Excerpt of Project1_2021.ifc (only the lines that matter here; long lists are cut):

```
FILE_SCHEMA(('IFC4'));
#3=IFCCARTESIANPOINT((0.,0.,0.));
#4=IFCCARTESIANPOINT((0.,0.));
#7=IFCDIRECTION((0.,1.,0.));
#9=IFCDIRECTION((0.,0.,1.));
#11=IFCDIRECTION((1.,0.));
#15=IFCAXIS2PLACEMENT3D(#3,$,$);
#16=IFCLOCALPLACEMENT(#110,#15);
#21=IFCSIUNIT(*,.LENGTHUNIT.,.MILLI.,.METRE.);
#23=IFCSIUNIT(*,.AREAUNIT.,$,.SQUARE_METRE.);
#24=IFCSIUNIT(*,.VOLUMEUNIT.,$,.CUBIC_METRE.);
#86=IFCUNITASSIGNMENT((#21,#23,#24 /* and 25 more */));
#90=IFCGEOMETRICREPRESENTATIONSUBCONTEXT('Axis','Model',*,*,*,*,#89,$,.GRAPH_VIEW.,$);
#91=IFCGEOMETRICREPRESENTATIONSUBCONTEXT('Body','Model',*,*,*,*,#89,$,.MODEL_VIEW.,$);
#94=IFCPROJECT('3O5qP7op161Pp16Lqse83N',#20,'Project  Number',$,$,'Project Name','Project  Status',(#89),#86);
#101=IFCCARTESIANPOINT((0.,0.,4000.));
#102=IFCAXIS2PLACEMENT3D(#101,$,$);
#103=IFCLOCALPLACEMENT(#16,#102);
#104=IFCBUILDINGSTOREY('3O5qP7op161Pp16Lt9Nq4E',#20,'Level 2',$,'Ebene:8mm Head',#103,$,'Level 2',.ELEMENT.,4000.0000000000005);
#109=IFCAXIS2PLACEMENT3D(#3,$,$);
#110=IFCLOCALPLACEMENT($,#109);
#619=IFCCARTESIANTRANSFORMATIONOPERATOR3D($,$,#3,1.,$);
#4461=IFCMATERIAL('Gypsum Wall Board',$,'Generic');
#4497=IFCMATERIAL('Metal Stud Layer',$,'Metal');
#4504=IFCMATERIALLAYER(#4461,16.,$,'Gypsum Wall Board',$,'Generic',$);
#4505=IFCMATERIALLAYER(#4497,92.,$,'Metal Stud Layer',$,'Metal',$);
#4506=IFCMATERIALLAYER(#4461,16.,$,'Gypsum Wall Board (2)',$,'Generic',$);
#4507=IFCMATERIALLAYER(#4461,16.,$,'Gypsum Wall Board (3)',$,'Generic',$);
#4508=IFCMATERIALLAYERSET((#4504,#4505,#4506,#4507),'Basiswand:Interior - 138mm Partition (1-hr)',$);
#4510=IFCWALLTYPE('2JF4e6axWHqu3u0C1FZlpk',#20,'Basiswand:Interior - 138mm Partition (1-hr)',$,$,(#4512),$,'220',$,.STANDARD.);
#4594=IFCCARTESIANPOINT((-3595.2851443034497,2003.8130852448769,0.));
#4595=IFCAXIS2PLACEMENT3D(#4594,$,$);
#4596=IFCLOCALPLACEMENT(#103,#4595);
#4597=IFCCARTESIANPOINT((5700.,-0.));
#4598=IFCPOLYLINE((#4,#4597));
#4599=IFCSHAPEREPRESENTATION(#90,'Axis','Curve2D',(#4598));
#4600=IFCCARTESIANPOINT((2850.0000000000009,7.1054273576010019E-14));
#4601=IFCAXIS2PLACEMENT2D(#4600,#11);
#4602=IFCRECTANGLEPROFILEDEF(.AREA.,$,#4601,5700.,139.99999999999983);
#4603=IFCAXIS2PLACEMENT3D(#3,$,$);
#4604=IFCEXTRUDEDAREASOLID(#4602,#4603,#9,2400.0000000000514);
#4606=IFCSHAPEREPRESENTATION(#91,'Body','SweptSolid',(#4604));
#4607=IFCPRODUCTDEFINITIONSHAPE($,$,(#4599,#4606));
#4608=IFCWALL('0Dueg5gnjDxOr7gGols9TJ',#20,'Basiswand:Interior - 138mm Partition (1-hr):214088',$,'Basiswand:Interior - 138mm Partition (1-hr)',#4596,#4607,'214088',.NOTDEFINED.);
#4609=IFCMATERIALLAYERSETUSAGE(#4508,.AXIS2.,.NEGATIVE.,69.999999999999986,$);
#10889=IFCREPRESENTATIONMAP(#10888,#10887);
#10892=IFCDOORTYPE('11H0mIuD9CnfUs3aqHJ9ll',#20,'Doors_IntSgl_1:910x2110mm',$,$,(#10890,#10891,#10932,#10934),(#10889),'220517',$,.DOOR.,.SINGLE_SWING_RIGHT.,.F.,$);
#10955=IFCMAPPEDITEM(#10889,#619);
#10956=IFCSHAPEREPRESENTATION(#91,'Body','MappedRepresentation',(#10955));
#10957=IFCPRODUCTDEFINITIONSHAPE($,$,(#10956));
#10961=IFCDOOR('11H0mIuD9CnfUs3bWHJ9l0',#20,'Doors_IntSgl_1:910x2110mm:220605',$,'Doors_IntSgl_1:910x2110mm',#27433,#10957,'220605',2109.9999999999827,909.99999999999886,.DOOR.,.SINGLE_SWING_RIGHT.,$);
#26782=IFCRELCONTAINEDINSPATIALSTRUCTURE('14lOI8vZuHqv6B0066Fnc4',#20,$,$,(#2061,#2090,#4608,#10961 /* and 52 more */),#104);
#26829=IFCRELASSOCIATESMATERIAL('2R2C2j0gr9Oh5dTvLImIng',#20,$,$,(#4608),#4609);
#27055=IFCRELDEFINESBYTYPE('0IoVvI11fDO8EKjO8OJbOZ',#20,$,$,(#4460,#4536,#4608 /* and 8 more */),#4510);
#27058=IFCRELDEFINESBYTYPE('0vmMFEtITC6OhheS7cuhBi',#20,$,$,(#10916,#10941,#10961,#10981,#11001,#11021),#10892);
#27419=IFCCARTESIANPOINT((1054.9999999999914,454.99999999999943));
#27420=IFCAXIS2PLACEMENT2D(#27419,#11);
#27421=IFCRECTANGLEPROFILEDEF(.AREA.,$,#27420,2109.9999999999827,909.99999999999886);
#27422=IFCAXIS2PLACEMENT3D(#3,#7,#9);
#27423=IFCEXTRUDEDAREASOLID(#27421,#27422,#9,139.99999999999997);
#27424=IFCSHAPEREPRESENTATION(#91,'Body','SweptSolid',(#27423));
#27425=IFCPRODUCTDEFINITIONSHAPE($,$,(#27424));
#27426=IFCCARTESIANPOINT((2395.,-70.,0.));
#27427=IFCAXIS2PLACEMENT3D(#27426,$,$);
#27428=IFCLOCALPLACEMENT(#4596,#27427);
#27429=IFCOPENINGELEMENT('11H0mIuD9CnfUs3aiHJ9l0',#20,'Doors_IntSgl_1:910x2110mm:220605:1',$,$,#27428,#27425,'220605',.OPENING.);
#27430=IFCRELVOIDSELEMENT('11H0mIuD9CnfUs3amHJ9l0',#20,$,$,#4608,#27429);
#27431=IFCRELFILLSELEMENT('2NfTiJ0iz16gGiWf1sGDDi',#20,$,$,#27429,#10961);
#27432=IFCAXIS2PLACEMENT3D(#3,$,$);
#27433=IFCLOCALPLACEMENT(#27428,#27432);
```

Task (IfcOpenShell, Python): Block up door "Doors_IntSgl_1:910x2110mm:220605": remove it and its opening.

```python
import ifcopenshell
import ifcopenshell.api.feature
import ifcopenshell.api.root
import ifcopenshell.geom
import ifcopenshell.util.shape

model = ifcopenshell.open("Project1_2021.ifc")
settings = ifcopenshell.geom.settings()


def volume(element):
    """Net volume in cubic metres, openings subtracted."""
    shape = ifcopenshell.geom.create_shape(settings, element)
    return ifcopenshell.util.shape.get_volume(shape.geometry)


door = model.by_guid("11H0mIuD9CnfUs3bWHJ9l0")
opening = door.FillsVoids[0].RelatingOpeningElement
wall = opening.VoidsElements[0].RelatingBuildingElement
before = volume(wall)

ifcopenshell.api.root.remove_product(model, product=door)
ifcopenshell.api.feature.remove_feature(model, feature=opening)

after = volume(wall)

print(f"wall volume {before:.3f} -> {after:.3f} m3")

model.write("Project1_2021_edited.ifc")
```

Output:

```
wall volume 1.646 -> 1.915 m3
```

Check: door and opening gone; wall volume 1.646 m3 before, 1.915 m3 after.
